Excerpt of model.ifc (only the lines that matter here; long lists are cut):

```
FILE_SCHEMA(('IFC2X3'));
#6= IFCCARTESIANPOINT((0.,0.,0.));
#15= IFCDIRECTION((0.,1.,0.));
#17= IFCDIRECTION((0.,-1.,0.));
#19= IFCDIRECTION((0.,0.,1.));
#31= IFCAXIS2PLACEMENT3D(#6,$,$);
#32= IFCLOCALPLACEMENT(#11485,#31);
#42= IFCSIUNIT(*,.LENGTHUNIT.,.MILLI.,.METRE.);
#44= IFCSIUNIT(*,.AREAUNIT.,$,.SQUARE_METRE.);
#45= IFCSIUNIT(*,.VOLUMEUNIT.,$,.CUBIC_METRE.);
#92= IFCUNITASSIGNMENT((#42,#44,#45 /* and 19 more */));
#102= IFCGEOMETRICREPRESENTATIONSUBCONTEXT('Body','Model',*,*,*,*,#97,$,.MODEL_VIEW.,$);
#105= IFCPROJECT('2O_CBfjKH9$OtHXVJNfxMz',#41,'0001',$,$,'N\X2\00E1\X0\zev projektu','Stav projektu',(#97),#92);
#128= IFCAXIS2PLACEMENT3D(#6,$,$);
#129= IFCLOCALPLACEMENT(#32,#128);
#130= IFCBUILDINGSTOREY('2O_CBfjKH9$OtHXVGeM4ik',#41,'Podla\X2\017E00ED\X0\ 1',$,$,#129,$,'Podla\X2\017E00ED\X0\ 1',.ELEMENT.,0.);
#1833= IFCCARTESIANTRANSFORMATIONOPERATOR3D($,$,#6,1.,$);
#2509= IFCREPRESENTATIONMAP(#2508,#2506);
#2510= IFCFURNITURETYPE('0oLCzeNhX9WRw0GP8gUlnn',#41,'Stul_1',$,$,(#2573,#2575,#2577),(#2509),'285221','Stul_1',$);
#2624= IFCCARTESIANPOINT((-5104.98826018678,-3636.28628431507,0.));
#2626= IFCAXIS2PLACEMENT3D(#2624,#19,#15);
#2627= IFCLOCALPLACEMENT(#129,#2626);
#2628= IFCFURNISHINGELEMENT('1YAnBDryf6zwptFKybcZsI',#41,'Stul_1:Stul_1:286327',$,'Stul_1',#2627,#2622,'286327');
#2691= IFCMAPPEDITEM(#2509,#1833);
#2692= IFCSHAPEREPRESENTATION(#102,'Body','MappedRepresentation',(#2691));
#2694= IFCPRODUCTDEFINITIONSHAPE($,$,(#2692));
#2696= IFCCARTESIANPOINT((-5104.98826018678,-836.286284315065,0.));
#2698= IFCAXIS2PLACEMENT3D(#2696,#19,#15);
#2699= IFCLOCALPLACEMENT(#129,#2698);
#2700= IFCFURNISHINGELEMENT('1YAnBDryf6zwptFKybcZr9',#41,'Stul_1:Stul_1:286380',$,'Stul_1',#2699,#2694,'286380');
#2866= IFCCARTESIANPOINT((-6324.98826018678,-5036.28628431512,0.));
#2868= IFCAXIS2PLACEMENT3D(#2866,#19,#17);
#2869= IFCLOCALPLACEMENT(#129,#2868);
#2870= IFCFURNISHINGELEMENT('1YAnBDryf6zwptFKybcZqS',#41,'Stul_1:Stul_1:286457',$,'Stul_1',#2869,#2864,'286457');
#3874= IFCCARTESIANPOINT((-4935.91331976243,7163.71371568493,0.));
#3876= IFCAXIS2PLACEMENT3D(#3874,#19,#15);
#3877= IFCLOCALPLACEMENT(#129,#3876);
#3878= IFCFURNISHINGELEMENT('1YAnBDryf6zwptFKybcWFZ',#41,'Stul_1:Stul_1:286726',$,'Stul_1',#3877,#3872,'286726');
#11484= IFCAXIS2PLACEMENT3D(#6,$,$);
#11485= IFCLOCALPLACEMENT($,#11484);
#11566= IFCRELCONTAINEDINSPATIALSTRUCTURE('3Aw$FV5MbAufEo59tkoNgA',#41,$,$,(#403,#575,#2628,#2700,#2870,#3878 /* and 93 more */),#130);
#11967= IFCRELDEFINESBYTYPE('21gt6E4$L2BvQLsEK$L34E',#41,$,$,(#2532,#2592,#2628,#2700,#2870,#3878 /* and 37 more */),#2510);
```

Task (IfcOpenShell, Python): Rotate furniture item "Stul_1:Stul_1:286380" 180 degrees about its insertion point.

```python
import ifcopenshell
import ifcopenshell.api.geometry
import ifcopenshell.util.placement

model = ifcopenshell.open("model.ifc")

item = model.by_guid("1YAnBDryf6zwptFKybcZr9")
matrix = ifcopenshell.util.placement.get_local_placement(item.ObjectPlacement)
matrix = matrix @ ifcopenshell.util.placement.rotation(180, "Z")
ifcopenshell.api.geometry.edit_object_placement(model, product=item, matrix=matrix, is_si=False)

print(ifcopenshell.util.placement.get_local_placement(item.ObjectPlacement).round(3) + 0.0)

model.write("model_updated.ifc")
```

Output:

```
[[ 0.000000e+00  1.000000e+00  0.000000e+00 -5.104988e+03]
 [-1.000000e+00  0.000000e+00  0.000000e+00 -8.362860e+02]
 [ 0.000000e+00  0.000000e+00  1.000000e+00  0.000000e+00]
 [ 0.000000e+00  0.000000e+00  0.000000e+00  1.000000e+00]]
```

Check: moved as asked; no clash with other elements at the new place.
